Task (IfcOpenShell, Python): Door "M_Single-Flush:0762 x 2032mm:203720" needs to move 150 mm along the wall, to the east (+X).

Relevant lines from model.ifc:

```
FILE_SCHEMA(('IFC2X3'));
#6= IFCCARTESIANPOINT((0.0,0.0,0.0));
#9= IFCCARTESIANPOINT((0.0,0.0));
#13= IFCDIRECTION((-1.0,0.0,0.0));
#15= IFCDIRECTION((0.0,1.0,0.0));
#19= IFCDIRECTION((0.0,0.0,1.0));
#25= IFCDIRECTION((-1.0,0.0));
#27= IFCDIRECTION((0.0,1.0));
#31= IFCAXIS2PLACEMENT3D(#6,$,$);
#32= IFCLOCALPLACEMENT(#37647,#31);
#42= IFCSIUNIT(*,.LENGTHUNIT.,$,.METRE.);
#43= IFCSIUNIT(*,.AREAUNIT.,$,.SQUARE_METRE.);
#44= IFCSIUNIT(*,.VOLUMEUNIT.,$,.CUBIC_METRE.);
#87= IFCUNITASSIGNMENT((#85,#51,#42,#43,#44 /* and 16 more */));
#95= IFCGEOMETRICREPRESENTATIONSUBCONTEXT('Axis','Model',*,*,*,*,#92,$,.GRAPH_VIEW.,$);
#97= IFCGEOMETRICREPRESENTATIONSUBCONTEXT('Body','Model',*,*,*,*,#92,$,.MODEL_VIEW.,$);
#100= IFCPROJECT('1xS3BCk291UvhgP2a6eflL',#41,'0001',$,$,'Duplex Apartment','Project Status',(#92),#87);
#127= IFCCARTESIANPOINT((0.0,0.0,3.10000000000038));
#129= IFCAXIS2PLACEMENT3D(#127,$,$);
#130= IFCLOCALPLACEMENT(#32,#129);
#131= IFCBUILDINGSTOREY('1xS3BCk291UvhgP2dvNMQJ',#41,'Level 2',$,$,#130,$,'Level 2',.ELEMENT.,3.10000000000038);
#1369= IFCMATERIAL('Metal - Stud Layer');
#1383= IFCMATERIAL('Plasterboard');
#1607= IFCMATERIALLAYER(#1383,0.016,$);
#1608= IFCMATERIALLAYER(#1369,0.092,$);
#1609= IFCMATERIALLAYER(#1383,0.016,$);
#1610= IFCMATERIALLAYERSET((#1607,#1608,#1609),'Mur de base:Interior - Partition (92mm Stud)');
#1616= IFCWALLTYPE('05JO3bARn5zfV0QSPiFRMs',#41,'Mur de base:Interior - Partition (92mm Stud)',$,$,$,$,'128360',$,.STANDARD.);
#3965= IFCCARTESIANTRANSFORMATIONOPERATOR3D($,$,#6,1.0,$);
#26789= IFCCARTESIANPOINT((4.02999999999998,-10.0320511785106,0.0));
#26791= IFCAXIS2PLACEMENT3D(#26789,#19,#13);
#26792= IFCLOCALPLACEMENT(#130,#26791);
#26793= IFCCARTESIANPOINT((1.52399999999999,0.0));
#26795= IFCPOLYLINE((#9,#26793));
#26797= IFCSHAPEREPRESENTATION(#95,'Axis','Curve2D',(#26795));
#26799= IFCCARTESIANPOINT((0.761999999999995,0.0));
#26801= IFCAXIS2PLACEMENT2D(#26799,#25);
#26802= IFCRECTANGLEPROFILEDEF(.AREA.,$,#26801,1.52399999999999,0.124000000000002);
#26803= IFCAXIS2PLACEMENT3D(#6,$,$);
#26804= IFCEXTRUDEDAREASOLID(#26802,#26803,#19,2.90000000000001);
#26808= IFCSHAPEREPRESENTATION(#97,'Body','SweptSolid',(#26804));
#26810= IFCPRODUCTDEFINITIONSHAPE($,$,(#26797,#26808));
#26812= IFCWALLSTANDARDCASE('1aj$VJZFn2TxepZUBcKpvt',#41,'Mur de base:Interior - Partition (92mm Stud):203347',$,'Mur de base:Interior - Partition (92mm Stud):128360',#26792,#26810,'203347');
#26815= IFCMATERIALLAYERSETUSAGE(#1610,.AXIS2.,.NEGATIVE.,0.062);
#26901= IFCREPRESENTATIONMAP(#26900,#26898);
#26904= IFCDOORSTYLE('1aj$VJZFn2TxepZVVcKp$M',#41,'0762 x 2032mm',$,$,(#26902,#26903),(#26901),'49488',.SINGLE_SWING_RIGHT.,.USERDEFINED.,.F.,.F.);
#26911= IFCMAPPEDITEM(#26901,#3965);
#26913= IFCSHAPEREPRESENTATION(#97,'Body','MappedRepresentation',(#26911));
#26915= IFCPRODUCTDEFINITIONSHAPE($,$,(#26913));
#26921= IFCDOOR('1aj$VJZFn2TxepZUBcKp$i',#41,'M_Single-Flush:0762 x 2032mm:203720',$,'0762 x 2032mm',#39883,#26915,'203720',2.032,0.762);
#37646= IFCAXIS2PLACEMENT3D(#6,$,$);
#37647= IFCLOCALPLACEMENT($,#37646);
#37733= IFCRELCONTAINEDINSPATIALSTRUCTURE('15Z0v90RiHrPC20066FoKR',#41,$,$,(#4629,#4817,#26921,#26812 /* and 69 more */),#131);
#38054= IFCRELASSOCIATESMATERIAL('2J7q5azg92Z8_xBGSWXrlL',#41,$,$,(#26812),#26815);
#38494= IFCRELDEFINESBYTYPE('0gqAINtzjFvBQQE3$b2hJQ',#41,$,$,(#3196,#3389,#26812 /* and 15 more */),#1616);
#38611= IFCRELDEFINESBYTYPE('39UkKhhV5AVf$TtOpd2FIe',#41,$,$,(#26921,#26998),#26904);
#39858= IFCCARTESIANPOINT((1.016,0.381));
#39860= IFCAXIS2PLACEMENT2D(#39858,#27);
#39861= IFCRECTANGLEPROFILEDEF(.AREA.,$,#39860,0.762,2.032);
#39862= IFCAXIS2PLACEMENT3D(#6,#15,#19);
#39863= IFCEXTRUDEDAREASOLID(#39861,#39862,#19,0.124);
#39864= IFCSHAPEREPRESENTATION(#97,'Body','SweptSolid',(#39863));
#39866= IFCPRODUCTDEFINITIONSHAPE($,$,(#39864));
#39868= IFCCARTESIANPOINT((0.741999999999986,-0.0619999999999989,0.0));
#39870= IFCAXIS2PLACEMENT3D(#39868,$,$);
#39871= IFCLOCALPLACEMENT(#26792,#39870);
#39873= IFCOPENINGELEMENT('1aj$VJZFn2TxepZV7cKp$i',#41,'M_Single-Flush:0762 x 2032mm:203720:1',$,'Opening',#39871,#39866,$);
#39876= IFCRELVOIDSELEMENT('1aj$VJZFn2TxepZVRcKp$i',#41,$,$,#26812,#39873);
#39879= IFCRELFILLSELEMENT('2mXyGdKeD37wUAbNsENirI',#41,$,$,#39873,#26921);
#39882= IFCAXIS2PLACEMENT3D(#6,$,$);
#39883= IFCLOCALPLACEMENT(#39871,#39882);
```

```python
import ifcopenshell
import ifcopenshell.api.geometry
import ifcopenshell.util.placement
import ifcopenshell.util.unit

model = ifcopenshell.open("model.ifc")
unit_scale = ifcopenshell.util.unit.calculate_unit_scale(model)

door = model.by_guid("1aj$VJZFn2TxepZUBcKp$i")
opening = door.FillsVoids[0].RelatingOpeningElement
wall = opening.VoidsElements[0].RelatingBuildingElement

wall_matrix = ifcopenshell.util.placement.get_local_placement(wall.ObjectPlacement)
shift = wall_matrix[:3, 0] * -0.15 / unit_scale
before = ifcopenshell.util.placement.get_local_placement(door.ObjectPlacement)[:3, 3].copy()

# The door is placed relative to its opening, so it follows when the opening moves.
matrix = ifcopenshell.util.placement.get_local_placement(opening.ObjectPlacement)
matrix[:3, 3] += shift
ifcopenshell.api.geometry.edit_object_placement(
    model, product=opening, matrix=matrix, is_si=False, should_transform_children=True
)

after = ifcopenshell.util.placement.get_local_placement(door.ObjectPlacement)[:3, 3]
print("door moved by", (after - before).round(3) + 0.0)

model.write("model_rev.ifc")
```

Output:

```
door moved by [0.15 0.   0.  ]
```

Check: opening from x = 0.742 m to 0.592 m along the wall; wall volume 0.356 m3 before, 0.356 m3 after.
